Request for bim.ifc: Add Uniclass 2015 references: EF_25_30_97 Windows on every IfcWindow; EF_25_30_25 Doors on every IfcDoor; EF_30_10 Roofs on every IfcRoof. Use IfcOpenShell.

First a look at what the model holds.

```python
import ifcopenshell

model = ifcopenshell.open("bim.ifc")
print(model.schema)
print("classifications:", [c.Name for c in model.by_type("IfcClassification")])
for ifc_class in ("IfcDoor", "IfcRoof", "IfcStair", "IfcWall", "IfcWindow"):
    print(ifc_class, len(model.by_type(ifc_class)))
```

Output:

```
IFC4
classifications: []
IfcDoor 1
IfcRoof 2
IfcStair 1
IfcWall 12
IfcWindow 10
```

```python
import ifcopenshell
import ifcopenshell.api.classification

model = ifcopenshell.open("bim.ifc")

system = ifcopenshell.api.classification.add_classification(model, classification="Uniclass 2015")

codes = {
    "IfcWindow": ("EF_25_30_97", "Windows"),
    "IfcDoor": ("EF_25_30_25", "Doors"),
    "IfcRoof": ("EF_30_10", "Roofs"),
}
for ifc_class, (code, name) in codes.items():
    products = model.by_type(ifc_class)
    ifcopenshell.api.classification.add_reference(
        model, products=products, classification=system, identification=code, name=name
    )
    print(code, len(products))

model.write("bim-out.ifc")
```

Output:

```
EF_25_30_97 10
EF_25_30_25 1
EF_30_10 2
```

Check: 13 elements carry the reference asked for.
